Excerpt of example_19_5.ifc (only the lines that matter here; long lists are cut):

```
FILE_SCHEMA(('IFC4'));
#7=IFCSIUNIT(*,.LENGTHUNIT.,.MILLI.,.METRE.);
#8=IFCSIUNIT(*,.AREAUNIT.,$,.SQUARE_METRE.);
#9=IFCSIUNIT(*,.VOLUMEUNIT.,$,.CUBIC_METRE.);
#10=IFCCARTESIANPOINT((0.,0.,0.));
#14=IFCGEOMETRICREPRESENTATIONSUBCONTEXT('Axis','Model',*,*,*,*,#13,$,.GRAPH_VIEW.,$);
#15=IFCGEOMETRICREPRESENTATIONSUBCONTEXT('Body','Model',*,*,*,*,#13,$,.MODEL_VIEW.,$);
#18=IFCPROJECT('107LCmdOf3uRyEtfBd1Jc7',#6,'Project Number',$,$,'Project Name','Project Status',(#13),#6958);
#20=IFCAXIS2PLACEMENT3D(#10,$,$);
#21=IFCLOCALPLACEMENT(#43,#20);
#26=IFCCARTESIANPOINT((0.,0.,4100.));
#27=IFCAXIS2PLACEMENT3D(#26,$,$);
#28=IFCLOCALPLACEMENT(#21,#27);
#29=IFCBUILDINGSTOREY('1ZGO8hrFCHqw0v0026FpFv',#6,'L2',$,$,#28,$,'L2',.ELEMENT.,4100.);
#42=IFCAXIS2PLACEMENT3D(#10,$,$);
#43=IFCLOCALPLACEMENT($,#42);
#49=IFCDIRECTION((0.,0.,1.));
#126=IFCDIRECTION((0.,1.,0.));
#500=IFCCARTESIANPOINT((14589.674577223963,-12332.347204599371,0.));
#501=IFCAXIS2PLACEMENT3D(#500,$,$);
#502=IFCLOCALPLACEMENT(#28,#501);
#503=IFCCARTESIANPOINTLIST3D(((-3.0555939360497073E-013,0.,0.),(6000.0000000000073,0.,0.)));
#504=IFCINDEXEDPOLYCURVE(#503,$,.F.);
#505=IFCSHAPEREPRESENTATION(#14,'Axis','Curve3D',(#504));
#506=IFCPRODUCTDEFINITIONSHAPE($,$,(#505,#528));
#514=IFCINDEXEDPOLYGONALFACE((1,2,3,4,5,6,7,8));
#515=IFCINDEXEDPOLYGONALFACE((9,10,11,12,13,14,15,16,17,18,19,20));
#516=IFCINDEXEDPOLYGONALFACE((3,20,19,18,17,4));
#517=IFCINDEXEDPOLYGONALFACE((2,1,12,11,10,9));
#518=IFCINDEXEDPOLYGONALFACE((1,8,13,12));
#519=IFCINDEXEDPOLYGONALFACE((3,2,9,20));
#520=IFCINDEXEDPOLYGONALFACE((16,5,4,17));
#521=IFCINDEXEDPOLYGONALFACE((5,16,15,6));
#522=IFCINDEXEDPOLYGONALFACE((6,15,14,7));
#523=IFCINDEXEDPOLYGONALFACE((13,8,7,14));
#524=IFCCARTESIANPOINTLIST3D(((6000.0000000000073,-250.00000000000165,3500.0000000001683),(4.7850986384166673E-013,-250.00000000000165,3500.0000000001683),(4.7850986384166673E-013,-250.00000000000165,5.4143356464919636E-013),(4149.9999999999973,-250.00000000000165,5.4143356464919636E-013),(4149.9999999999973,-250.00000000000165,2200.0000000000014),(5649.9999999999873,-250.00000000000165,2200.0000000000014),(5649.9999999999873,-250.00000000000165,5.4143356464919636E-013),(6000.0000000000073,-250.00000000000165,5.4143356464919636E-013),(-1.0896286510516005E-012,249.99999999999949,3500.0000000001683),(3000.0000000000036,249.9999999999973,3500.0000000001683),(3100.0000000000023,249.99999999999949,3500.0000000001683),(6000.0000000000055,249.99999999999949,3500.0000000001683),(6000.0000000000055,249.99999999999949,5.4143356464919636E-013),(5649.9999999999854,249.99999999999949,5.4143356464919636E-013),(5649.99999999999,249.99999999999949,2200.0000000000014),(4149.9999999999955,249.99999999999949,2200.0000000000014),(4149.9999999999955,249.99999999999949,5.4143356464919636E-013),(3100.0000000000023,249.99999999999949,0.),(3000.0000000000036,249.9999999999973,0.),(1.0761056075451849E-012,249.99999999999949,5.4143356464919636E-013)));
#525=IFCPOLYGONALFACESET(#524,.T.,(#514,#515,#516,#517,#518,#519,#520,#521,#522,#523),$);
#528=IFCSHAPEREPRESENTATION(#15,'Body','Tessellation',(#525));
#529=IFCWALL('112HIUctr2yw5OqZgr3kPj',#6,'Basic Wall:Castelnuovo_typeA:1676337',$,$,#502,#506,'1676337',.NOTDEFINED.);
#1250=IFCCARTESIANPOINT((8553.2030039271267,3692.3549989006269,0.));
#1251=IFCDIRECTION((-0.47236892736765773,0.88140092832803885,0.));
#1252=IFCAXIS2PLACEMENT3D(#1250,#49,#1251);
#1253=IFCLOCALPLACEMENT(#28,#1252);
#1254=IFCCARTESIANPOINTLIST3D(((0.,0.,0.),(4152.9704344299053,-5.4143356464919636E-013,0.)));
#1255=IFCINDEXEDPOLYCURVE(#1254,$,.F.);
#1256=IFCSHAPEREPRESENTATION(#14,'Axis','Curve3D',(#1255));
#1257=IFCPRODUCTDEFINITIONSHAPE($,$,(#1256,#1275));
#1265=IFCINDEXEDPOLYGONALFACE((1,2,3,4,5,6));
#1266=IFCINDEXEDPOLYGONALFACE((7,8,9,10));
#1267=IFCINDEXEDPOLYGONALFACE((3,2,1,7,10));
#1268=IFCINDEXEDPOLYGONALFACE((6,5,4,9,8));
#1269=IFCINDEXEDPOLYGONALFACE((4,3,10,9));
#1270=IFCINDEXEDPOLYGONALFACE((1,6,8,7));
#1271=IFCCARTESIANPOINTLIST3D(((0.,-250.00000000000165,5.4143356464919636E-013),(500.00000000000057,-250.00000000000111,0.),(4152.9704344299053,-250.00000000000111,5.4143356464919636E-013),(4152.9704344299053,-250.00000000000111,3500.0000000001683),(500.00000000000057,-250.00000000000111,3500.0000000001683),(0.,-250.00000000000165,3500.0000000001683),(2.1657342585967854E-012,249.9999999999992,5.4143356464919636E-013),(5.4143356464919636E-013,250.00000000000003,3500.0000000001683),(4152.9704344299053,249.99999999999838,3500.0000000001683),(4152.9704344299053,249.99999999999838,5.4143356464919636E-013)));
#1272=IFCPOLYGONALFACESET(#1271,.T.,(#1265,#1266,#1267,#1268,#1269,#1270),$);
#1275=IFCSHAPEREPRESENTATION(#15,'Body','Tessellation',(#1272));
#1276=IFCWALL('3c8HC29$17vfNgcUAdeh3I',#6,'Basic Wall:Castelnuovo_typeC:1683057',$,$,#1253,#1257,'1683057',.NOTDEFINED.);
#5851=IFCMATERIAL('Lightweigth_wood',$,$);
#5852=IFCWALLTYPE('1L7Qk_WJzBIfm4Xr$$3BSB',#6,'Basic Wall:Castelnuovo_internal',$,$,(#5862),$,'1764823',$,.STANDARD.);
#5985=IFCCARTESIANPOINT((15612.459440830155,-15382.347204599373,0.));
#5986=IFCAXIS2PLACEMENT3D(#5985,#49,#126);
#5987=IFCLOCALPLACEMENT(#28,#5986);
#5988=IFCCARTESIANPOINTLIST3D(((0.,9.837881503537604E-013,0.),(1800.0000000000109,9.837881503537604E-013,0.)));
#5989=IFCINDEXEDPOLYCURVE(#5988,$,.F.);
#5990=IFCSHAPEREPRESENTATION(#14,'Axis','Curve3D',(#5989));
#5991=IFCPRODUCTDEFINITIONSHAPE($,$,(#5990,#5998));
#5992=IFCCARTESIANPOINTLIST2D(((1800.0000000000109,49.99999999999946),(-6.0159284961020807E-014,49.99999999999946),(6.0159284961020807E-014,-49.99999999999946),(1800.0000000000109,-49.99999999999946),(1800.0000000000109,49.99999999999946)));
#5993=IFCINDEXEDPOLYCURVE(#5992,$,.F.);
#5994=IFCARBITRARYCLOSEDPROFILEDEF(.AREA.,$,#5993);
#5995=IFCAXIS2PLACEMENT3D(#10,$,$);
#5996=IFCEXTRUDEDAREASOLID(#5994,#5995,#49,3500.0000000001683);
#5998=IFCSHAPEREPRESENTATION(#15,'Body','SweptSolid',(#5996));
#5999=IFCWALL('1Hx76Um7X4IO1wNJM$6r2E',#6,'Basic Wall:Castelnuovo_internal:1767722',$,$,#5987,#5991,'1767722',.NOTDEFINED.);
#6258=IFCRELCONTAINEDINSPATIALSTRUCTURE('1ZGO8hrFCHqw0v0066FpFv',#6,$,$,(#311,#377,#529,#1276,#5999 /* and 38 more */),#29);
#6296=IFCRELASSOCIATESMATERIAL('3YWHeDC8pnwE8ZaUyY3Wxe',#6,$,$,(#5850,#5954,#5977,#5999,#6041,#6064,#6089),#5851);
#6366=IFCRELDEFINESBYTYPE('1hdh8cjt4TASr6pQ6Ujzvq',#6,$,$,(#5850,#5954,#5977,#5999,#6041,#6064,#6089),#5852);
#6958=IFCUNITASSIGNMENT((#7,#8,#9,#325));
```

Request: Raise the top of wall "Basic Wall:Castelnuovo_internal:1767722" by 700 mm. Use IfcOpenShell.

```python
import ifcopenshell
import ifcopenshell.geom
import ifcopenshell.util.representation
import ifcopenshell.util.shape
import ifcopenshell.util.unit

model = ifcopenshell.open("example_19_5.ifc")
unit_scale = ifcopenshell.util.unit.calculate_unit_scale(model)
settings = ifcopenshell.geom.settings()


def volume(element):
    """Net volume in cubic metres, openings subtracted."""
    shape = ifcopenshell.geom.create_shape(settings, element)
    return ifcopenshell.util.shape.get_volume(shape.geometry)


wall = model.by_guid("1Hx76Um7X4IO1wNJM$6r2E")
before = volume(wall)

body = ifcopenshell.util.representation.get_representation(wall, "Model", "Body")
solid = body.Items[0]
old_height = solid.Depth
solid.Depth += 0.7 / unit_scale
after = volume(wall)

print(f"height {old_height:g} -> {solid.Depth:g}, volume {before:.3f} -> {after:.3f} m3")

model.write("example_19_5-out.ifc")
```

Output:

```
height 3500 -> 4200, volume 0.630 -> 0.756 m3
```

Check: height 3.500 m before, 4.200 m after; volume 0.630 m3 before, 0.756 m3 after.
